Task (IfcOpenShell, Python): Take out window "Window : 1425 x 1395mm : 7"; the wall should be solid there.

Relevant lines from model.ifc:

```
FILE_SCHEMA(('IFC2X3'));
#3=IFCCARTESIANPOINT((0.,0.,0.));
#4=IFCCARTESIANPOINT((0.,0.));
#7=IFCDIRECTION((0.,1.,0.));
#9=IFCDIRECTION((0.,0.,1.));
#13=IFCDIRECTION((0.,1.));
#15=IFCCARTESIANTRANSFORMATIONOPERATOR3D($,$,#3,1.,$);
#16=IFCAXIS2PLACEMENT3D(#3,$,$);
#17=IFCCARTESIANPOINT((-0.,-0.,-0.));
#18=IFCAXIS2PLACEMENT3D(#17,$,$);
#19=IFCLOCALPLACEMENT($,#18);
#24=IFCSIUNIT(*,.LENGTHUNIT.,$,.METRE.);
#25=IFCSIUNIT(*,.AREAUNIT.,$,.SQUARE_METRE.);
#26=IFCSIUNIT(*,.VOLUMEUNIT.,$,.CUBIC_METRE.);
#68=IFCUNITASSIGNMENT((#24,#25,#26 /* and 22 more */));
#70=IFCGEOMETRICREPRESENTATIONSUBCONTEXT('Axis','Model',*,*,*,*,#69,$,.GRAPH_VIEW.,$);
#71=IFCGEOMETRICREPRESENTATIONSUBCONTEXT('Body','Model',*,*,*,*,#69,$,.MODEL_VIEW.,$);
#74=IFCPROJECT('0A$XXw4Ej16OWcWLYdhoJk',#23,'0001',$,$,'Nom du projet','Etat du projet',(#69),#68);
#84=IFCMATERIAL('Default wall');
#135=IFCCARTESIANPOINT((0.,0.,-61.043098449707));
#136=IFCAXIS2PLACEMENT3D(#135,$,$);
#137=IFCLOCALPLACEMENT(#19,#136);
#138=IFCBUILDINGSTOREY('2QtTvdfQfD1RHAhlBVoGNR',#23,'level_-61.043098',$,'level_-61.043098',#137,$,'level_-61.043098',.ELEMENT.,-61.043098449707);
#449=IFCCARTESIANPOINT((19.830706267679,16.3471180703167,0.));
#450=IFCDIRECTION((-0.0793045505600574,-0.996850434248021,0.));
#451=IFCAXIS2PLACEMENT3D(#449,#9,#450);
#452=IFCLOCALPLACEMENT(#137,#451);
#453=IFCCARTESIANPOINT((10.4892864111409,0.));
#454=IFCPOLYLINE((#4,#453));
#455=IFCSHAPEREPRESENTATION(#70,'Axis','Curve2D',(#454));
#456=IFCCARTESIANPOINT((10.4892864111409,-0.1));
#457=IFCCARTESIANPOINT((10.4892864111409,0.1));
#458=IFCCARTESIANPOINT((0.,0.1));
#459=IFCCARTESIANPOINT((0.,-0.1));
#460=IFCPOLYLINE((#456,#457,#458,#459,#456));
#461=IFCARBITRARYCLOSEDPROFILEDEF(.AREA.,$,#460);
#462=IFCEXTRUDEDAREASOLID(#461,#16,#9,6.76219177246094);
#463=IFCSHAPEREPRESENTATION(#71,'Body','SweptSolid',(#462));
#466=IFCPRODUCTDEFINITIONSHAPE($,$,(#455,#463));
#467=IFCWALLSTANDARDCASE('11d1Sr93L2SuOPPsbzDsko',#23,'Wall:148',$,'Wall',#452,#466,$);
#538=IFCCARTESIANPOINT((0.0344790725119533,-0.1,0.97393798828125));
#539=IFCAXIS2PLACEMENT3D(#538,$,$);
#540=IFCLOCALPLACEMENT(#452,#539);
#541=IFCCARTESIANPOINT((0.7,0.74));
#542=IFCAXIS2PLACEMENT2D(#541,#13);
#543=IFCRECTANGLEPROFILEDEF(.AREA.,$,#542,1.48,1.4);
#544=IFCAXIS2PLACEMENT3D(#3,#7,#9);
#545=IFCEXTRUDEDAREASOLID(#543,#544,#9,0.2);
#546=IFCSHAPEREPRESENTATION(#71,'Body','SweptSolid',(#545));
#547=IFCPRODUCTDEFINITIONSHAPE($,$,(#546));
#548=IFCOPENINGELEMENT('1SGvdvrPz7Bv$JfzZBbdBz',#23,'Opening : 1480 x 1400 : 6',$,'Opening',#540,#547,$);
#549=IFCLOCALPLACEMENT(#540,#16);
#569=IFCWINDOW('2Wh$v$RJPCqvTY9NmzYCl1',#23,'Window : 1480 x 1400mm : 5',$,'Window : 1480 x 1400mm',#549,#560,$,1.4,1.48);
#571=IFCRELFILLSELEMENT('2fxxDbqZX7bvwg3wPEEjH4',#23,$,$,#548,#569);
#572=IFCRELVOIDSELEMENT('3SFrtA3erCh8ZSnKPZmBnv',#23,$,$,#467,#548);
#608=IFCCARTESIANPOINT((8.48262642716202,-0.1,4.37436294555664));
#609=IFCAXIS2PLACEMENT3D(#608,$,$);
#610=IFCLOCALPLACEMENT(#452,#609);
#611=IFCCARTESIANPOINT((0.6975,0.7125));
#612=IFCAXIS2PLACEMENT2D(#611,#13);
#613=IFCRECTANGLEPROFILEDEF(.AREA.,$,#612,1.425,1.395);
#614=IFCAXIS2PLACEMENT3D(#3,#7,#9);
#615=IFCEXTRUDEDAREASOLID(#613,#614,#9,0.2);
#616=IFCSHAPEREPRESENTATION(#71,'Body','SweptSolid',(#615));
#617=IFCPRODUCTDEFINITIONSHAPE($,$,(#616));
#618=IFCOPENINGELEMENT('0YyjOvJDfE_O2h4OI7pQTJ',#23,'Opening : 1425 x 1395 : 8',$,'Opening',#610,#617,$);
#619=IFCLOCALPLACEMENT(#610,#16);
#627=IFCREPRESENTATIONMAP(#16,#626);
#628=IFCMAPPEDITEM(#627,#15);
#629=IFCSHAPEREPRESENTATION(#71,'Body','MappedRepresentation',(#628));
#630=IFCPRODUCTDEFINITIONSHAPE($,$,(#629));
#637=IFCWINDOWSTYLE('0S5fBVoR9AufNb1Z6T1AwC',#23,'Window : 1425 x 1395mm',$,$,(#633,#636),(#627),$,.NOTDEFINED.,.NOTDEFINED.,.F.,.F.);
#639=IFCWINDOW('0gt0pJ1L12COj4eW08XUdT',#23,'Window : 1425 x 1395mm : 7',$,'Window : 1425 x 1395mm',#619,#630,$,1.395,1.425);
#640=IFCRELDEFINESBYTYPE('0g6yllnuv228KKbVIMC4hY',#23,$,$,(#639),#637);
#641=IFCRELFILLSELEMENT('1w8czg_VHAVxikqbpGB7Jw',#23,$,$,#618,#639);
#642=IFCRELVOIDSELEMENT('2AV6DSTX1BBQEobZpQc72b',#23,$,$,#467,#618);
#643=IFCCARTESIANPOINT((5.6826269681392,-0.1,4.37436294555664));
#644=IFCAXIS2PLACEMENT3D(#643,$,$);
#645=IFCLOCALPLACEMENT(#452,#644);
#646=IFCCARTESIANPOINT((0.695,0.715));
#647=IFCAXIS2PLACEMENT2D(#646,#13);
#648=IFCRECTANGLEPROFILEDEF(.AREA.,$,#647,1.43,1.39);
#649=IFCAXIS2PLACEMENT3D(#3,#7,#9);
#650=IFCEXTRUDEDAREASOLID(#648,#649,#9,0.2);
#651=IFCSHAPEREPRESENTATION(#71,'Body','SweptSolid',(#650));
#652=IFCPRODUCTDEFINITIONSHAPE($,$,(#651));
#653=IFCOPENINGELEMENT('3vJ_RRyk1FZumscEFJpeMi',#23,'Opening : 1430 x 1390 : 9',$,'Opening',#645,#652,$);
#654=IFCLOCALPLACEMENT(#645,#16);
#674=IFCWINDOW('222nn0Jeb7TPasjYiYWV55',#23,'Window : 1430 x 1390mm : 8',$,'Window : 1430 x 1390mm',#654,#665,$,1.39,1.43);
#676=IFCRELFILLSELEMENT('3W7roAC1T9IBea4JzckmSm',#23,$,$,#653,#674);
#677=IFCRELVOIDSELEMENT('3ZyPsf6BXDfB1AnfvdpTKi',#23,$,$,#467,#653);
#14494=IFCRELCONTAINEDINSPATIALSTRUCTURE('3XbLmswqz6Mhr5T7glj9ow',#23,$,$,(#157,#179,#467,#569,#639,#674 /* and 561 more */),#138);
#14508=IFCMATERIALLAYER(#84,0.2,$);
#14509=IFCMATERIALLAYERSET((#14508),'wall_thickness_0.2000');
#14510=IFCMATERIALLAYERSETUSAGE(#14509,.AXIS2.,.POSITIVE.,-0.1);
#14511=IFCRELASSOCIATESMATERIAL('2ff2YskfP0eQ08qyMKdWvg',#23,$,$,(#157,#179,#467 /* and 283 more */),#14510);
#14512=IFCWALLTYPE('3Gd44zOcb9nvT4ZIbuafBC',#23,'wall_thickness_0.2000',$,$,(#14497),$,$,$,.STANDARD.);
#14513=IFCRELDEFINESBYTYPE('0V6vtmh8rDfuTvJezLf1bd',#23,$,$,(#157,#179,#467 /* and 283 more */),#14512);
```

```python
import ifcopenshell
import ifcopenshell.api.feature
import ifcopenshell.api.root
import ifcopenshell.geom
import ifcopenshell.util.shape

model = ifcopenshell.open("model.ifc")
settings = ifcopenshell.geom.settings()


def volume(element):
    """Net volume in cubic metres, openings subtracted."""
    shape = ifcopenshell.geom.create_shape(settings, element)
    return ifcopenshell.util.shape.get_volume(shape.geometry)


window = model.by_guid("0gt0pJ1L12COj4eW08XUdT")
opening = window.FillsVoids[0].RelatingOpeningElement
wall = opening.VoidsElements[0].RelatingBuildingElement
before = volume(wall)

ifcopenshell.api.root.remove_product(model, product=window)
ifcopenshell.api.feature.remove_feature(model, feature=opening)

after = volume(wall)

print(f"wall volume {before:.3f} -> {after:.3f} m3")

model.write("model_updated.ifc")
```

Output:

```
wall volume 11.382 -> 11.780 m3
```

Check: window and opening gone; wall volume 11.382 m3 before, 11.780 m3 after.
